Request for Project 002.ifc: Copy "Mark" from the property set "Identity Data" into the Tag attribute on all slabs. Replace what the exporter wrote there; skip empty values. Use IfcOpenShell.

First a look at what the model holds.

```python
import ifcopenshell
import ifcopenshell.util.element

model = ifcopenshell.open("Project 002.ifc")
print(model.schema)
slabs = model.by_type("IfcSlab")
print(len(slabs), "slabs")
for e in slabs[:8]:
    source = ifcopenshell.util.element.get_pset(e, "Identity Data", "Mark")
    target = e.Tag
    print(e.id(), repr(source), repr(target), sep=" | ")
```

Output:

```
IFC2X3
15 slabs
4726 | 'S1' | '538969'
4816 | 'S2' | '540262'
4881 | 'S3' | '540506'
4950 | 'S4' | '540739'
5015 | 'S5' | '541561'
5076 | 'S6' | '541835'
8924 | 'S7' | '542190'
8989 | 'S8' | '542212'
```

```python
import ifcopenshell
import ifcopenshell.util.element

model = ifcopenshell.open("Project 002.ifc")

count = 0
for e in model.by_type("IfcSlab"):
    value = ifcopenshell.util.element.get_pset(e, "Identity Data", "Mark")
    current = e.Tag
    if not value or not value.strip() or current == value:
        continue
    e.Tag = value
    count += 1

print(count, "slabs updated")

model.write("Project 002_updated.ifc")
```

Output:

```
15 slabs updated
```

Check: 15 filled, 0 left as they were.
